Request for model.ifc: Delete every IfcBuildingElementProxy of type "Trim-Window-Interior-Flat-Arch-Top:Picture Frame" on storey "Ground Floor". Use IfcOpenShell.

First a look at what the model holds.

```python
import ifcopenshell
import ifcopenshell.util.element

model = ifcopenshell.open("model.ifc")
print(model.schema)
storey = next(s for s in model.by_type("IfcBuildingStorey") if s.Name == "Ground Floor")
proxies = [e for e in ifcopenshell.util.element.get_decomposition(storey) if e.is_a("IfcBuildingElementProxy")]
seen = {}
for e in proxies:
    element_type = ifcopenshell.util.element.get_type(e)
    name = element_type.Name if element_type not in (None, e) else None
    seen[name] = seen.get(name, 0) + 1
for name, count in sorted(seen.items(), key=str):
    print(count, "x", name)
```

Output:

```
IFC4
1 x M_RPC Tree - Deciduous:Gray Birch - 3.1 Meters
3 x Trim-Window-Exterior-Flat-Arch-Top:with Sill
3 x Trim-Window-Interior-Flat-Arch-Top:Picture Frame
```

```python
import ifcopenshell
import ifcopenshell.api.root
import ifcopenshell.util.element

model = ifcopenshell.open("model.ifc")

storey = next(s for s in model.by_type("IfcBuildingStorey") if s.Name == "Ground Floor")
proxies = [e for e in ifcopenshell.util.element.get_decomposition(storey) if e.is_a("IfcBuildingElementProxy")]
targets = [e for e in proxies if (t := ifcopenshell.util.element.get_type(e)) not in (None, e) and t.Name == "Trim-Window-Interior-Flat-Arch-Top:Picture Frame"]

for e in targets:
    ifcopenshell.api.root.remove_product(model, product=e)
print(len(targets), "removed")

model.write("model_updated.ifc")
```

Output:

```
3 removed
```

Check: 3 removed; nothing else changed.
